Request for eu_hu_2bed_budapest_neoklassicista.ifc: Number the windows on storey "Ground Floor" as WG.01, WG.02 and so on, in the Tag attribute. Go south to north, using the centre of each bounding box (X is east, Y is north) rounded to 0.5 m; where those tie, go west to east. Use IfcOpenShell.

First a look at what the model holds.

```python
import ifcopenshell
import ifcopenshell.util.element
import ifcopenshell.util.placement

model = ifcopenshell.open("eu_hu_2bed_budapest_neoklassicista.ifc")
print(model.schema)
storey = next(s for s in model.by_type("IfcBuildingStorey") if s.Name == "Ground Floor")
windows = [e for e in ifcopenshell.util.element.get_decomposition(storey) if e.is_a("IfcWindow")]
for e in sorted(windows, key=lambda e: e.id()):
    origin = ifcopenshell.util.placement.get_local_placement(e.ObjectPlacement)[:3, 3]
    print(e.id(), e.Tag, e.Name, origin.round(2) + 0.0, sep=" | ")
```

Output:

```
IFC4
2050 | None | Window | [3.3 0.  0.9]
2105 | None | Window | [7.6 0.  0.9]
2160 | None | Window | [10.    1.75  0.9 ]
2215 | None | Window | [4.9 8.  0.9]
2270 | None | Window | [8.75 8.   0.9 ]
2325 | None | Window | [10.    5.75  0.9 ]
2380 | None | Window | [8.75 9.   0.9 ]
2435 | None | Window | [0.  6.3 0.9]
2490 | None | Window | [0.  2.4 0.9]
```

```python
import ifcopenshell
import ifcopenshell.geom
import ifcopenshell.util.element
import ifcopenshell.util.shape

model = ifcopenshell.open("eu_hu_2bed_budapest_neoklassicista.ifc")
settings = ifcopenshell.geom.settings()
settings.set("use-world-coords", True)


def centre(element):
    shape = ifcopenshell.geom.create_shape(settings, element)
    return ifcopenshell.util.shape.get_bbox_centroid(shape.geometry)


storey = next(s for s in model.by_type("IfcBuildingStorey") if s.Name == "Ground Floor")
windows = [e for e in ifcopenshell.util.element.get_decomposition(storey) if e.is_a("IfcWindow")]

# Insertion points can sit at a corner or the storey origin, so sort by the geometry (in metres).
centres = {e: centre(e) for e in windows}
windows.sort(key=lambda e: (round(centres[e][1] / 0.5), centres[e][0]))

for i, e in enumerate(windows, start=1):
    number = f"WG.{i:02d}"
    e.Tag = number
    print(e.id(), number)

model.write("eu_hu_2bed_budapest_neoklassicista-out.ifc")
```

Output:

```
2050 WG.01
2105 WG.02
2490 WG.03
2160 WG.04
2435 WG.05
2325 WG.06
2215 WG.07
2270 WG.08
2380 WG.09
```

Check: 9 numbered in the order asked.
